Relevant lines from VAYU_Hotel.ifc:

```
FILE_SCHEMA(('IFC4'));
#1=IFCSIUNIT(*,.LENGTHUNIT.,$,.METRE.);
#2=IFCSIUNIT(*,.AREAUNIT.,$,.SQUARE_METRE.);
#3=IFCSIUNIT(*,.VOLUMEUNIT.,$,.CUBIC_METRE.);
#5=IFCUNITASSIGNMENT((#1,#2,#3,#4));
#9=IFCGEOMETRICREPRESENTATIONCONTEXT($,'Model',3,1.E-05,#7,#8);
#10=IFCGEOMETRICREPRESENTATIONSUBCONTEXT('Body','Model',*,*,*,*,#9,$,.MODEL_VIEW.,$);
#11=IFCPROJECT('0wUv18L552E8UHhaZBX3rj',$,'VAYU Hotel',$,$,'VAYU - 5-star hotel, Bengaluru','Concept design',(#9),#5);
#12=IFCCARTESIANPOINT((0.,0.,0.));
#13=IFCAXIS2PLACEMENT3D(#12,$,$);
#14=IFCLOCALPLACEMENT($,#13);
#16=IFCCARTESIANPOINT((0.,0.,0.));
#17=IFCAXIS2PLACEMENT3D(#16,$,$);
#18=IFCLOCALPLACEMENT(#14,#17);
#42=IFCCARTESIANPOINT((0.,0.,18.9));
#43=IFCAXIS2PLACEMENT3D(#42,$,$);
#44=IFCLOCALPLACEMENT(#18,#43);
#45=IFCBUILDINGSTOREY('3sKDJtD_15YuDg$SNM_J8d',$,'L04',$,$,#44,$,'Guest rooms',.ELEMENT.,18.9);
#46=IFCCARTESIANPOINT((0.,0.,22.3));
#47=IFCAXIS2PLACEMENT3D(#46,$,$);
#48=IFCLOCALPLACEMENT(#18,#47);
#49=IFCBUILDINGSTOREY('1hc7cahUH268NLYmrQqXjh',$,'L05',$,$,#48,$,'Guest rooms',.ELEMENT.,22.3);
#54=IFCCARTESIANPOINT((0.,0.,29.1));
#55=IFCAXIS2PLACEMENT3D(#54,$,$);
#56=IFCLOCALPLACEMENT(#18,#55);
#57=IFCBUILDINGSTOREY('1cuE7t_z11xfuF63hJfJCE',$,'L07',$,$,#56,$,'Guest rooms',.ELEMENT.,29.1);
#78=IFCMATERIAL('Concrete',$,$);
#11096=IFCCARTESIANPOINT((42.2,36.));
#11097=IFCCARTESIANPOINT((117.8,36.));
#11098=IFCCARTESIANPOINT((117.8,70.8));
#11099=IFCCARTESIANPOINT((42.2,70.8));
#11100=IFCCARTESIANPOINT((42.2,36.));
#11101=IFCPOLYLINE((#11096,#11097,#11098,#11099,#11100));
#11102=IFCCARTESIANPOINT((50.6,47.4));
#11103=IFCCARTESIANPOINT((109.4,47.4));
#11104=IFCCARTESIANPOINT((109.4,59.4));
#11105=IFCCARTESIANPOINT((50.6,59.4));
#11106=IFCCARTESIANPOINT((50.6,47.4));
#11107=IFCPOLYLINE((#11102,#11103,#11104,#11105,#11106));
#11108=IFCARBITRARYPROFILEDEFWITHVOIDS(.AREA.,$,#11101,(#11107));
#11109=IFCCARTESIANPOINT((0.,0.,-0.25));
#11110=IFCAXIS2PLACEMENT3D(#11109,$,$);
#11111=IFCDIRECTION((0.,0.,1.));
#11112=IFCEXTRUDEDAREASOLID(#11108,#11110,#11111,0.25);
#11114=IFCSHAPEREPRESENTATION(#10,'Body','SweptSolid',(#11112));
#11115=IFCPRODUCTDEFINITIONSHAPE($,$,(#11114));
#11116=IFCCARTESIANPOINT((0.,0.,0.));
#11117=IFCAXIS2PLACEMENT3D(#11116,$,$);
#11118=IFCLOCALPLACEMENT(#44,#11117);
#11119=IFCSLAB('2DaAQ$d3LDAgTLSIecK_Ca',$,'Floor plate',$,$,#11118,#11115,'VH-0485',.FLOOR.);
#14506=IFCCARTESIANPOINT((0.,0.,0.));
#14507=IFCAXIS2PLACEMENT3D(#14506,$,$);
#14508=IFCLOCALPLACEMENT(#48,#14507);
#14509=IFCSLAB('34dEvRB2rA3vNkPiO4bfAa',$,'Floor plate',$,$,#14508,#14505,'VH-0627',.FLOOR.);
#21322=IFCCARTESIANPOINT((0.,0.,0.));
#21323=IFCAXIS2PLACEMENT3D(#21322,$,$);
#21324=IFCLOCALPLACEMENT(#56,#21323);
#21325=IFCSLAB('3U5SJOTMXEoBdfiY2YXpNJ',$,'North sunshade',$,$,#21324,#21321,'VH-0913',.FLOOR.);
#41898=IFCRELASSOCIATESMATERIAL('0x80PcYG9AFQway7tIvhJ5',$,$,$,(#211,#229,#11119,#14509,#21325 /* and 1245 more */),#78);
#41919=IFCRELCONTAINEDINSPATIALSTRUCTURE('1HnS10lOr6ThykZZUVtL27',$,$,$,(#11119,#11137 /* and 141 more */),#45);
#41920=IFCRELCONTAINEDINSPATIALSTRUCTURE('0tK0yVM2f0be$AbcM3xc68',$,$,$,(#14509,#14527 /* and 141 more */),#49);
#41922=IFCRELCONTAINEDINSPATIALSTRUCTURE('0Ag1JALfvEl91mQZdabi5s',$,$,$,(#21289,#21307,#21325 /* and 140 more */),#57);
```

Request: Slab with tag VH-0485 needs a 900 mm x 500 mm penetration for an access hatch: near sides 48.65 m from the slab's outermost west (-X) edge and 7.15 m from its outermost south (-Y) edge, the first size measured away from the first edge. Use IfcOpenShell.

```python
import numpy as np
import ifcopenshell
import ifcopenshell.api.feature
import ifcopenshell.api.geometry
import ifcopenshell.api.root
import ifcopenshell.geom
import ifcopenshell.util.placement
import ifcopenshell.util.representation
import ifcopenshell.util.shape
import ifcopenshell.util.unit

model = ifcopenshell.open("VAYU_Hotel.ifc")
unit_scale = ifcopenshell.util.unit.calculate_unit_scale(model)
settings = ifcopenshell.geom.settings()


def volume(element):
    """Net volume in cubic metres, openings subtracted."""
    shape = ifcopenshell.geom.create_shape(settings, element)
    return ifcopenshell.util.shape.get_volume(shape.geometry)


slab = model.by_id(11119)
before = volume(slab)

# Extent in the slab's own axes, in metres. The edges named are its -X and -Y sides.
slab_shape = ifcopenshell.geom.create_shape(settings, slab)
vertices = ifcopenshell.util.shape.get_vertices(slab_shape.geometry)
x_min, y_min, bottom = vertices.min(axis=0)
top = vertices[:, 2].max()

opening = ifcopenshell.api.root.create_entity(model, ifc_class="IfcOpeningElement", name="Access hatch opening", predefined_type="OPENING")
context = ifcopenshell.util.representation.get_context(model, "Model", "Body", "MODEL_VIEW")
width, depth = 0.9, 0.5
outline = [(0.0, 0.0), (width, 0.0), (width, depth), (0.0, depth), (0.0, 0.0)]
# Overshoot both faces by 50 mm so the cut is clean.
shape = ifcopenshell.api.geometry.add_slab_representation(
    model, context=context, depth=top - bottom + 0.1, polyline=outline
)
ifcopenshell.api.geometry.assign_representation(model, product=opening, representation=shape)

matrix = ifcopenshell.util.placement.get_local_placement(slab.ObjectPlacement)
matrix[:, 3] = matrix @ np.append(np.array([x_min + 48.65, y_min + 7.15, bottom - 0.05]) / unit_scale, 1.0)
ifcopenshell.api.geometry.edit_object_placement(model, product=opening, matrix=matrix, is_si=False)
ifcopenshell.api.feature.add_feature(model, feature=opening, element=slab)

after = volume(slab)

print(f"slab volume {before:.3f} -> {after:.3f} m3")

model.write("VAYU_Hotel_updated.ifc")
```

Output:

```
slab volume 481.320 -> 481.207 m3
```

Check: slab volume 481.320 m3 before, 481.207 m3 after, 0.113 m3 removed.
